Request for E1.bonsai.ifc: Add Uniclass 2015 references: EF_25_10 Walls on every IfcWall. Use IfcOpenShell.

First a look at what the model holds.

```python
import ifcopenshell

model = ifcopenshell.open("E1.bonsai.ifc")
print(model.schema)
print("classifications:", [c.Name for c in model.by_type("IfcClassification")])
for ifc_class in ("IfcDoor", "IfcRoof", "IfcStair", "IfcWall", "IfcWindow"):
    print(ifc_class, len(model.by_type(ifc_class)))
```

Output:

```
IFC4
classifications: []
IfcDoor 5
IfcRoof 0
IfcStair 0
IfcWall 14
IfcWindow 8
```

```python
import ifcopenshell
import ifcopenshell.api.classification

model = ifcopenshell.open("E1.bonsai.ifc")

system = ifcopenshell.api.classification.add_classification(model, classification="Uniclass 2015")

codes = {
    "IfcWall": ("EF_25_10", "Walls"),
}
for ifc_class, (code, name) in codes.items():
    products = model.by_type(ifc_class)
    ifcopenshell.api.classification.add_reference(
        model, products=products, classification=system, identification=code, name=name
    )
    print(code, len(products))

model.write("E1.bonsai_edited.ifc")
```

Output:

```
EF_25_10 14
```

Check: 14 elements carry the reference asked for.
